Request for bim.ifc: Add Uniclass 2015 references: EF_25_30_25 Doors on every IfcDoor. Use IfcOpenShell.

First a look at what the model holds.

```python
import ifcopenshell

model = ifcopenshell.open("bim.ifc")
print(model.schema)
print("classifications:", [c.Name for c in model.by_type("IfcClassification")])
for ifc_class in ("IfcDoor", "IfcRoof", "IfcStair", "IfcWall", "IfcWindow"):
    print(ifc_class, len(model.by_type(ifc_class)))
```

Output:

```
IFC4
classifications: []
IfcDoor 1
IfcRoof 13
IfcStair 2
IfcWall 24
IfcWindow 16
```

```python
import ifcopenshell
import ifcopenshell.api.classification

model = ifcopenshell.open("bim.ifc")

system = ifcopenshell.api.classification.add_classification(model, classification="Uniclass 2015")

codes = {
    "IfcDoor": ("EF_25_30_25", "Doors"),
}
for ifc_class, (code, name) in codes.items():
    products = model.by_type(ifc_class)
    ifcopenshell.api.classification.add_reference(
        model, products=products, classification=system, identification=code, name=name
    )
    print(code, len(products))

model.write("bim_updated.ifc")
```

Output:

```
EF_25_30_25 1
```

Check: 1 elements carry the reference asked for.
